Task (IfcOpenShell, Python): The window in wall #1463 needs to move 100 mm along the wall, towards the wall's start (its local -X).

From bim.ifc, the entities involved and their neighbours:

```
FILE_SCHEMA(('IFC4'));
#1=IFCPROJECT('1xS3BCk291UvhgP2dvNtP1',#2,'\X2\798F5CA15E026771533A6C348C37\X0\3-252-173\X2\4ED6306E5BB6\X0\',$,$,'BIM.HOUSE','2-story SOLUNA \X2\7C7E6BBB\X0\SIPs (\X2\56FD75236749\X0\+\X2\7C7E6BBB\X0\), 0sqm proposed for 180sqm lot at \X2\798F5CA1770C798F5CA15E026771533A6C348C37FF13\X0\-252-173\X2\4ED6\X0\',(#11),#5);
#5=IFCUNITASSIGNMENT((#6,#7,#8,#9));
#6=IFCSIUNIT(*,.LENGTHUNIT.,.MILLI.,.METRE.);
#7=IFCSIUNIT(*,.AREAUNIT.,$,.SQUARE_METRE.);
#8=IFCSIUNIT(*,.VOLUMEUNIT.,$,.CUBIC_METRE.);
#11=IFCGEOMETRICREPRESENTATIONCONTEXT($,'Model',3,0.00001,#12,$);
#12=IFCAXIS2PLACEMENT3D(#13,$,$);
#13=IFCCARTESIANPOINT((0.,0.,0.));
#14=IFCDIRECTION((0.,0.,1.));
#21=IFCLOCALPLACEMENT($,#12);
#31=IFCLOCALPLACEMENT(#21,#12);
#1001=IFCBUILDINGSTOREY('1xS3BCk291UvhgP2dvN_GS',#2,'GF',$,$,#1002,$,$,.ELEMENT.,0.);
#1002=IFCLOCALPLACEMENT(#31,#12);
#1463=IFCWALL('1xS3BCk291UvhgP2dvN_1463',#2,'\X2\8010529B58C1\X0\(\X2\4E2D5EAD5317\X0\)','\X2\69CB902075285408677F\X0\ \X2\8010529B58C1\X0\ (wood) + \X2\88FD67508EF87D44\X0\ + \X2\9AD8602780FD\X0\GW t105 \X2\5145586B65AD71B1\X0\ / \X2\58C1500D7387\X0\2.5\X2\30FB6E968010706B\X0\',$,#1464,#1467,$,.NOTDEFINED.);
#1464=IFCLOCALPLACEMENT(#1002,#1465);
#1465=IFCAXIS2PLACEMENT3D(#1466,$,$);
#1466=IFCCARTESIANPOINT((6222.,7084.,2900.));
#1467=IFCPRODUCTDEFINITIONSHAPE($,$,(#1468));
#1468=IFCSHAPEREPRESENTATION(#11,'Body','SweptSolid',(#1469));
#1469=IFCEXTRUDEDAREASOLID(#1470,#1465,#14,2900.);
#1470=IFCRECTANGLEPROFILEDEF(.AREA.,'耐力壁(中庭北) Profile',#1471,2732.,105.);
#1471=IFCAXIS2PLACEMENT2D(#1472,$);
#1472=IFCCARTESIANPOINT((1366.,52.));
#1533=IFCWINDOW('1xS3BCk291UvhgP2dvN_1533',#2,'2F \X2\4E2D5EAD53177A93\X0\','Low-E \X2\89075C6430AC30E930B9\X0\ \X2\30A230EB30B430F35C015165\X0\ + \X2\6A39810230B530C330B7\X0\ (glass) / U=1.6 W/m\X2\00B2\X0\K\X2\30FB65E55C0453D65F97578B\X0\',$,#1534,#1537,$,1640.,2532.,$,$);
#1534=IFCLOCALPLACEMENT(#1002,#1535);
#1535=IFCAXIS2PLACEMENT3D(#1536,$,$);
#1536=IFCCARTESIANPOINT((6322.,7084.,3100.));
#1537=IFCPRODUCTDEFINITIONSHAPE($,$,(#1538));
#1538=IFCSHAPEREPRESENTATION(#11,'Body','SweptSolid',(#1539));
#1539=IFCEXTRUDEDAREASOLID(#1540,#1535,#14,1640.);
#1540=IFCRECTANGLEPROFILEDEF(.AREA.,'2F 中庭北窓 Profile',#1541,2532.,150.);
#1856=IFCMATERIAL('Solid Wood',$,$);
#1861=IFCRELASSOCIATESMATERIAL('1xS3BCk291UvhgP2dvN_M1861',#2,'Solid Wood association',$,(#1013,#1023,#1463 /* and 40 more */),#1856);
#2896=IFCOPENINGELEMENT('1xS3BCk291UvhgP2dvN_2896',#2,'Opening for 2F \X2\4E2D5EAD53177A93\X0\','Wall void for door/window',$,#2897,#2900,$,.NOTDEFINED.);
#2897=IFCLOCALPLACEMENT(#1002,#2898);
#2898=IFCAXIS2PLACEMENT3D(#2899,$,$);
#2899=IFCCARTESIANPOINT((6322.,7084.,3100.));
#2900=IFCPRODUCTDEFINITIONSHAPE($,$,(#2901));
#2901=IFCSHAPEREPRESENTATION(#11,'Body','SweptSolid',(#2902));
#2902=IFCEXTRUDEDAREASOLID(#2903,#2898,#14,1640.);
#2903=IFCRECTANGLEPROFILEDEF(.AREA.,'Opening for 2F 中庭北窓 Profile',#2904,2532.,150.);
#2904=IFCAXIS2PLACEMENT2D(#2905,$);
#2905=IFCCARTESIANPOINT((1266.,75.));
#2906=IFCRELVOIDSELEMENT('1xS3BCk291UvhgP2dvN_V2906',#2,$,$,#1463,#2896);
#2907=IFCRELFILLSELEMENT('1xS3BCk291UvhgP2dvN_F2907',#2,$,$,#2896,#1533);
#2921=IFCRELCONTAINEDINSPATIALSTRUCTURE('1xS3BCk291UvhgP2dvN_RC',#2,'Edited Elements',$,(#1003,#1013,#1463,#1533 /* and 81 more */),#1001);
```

```python
import ifcopenshell
import ifcopenshell.api.geometry
import ifcopenshell.util.placement
import ifcopenshell.util.unit

model = ifcopenshell.open("bim.ifc")
unit_scale = ifcopenshell.util.unit.calculate_unit_scale(model)

window = model.by_id(1533)
opening = window.FillsVoids[0].RelatingOpeningElement
wall = opening.VoidsElements[0].RelatingBuildingElement

wall_matrix = ifcopenshell.util.placement.get_local_placement(wall.ObjectPlacement)
shift = wall_matrix[:3, 0] * -0.1 / unit_scale
before = ifcopenshell.util.placement.get_local_placement(window.ObjectPlacement)[:3, 3].copy()

# The window is not placed relative to its opening, so move both.
for product in (opening, window):
    matrix = ifcopenshell.util.placement.get_local_placement(product.ObjectPlacement)
    matrix[:3, 3] += shift
    ifcopenshell.api.geometry.edit_object_placement(model, product=product, matrix=matrix, is_si=False)

after = ifcopenshell.util.placement.get_local_placement(window.ObjectPlacement)[:3, 3]
print("window moved by", (after - before).round(3) + 0.0)

model.write("bim_edited.ifc")
```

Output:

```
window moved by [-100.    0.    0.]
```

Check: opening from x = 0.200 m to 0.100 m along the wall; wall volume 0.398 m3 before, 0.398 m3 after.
